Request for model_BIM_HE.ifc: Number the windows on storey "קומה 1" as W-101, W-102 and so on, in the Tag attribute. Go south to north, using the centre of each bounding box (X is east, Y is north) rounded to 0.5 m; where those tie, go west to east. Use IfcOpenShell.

First a look at what the model holds.

```python
import ifcopenshell
import ifcopenshell.util.element
import ifcopenshell.util.placement

model = ifcopenshell.open("model_BIM_HE.ifc")
print(model.schema)
storey = next(s for s in model.by_type("IfcBuildingStorey") if s.Name == "קומה 1")
windows = [e for e in ifcopenshell.util.element.get_decomposition(storey) if e.is_a("IfcWindow")]
for e in sorted(windows, key=lambda e: e.id()):
    origin = ifcopenshell.util.placement.get_local_placement(e.ObjectPlacement)[:3, 3]
    print(e.id(), e.Tag, e.Name, origin.round(2) + 0.0, sep=" | ")
```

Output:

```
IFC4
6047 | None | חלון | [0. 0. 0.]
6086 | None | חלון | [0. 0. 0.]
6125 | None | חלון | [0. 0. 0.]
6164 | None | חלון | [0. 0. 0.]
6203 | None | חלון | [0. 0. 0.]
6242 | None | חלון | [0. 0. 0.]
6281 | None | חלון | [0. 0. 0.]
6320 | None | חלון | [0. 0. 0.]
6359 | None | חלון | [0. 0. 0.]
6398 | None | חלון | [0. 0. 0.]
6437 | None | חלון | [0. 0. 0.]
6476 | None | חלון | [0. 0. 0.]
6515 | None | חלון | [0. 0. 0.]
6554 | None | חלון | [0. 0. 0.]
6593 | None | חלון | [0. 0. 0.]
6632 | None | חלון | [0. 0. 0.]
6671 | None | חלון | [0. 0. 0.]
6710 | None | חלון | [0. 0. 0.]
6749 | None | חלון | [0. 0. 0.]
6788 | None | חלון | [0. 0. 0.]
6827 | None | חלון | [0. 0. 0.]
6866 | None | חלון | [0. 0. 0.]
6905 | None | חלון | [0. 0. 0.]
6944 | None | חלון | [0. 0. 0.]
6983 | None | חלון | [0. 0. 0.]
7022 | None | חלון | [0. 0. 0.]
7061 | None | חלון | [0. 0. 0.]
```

```python
import ifcopenshell
import ifcopenshell.geom
import ifcopenshell.util.element
import ifcopenshell.util.shape

model = ifcopenshell.open("model_BIM_HE.ifc")
settings = ifcopenshell.geom.settings()
settings.set("use-world-coords", True)


def centre(element):
    shape = ifcopenshell.geom.create_shape(settings, element)
    return ifcopenshell.util.shape.get_bbox_centroid(shape.geometry)


storey = next(s for s in model.by_type("IfcBuildingStorey") if s.Name == "קומה 1")
windows = [e for e in ifcopenshell.util.element.get_decomposition(storey) if e.is_a("IfcWindow")]

# Insertion points can sit at a corner or the storey origin, so sort by the geometry (in metres).
centres = {e: centre(e) for e in windows}
windows.sort(key=lambda e: (round(centres[e][1] / 0.5), centres[e][0]))

for i, e in enumerate(windows, start=1):
    number = f"W-1{i:02d}"
    e.Tag = number
    print(e.id(), number)

model.write("model_BIM_HE_updated.ifc")
```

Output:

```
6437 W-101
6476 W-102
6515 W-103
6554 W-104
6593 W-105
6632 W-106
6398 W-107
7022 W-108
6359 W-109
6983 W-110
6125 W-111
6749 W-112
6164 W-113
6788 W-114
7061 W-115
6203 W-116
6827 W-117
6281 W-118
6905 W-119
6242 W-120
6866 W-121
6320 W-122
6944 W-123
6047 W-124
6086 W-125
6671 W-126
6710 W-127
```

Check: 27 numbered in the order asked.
